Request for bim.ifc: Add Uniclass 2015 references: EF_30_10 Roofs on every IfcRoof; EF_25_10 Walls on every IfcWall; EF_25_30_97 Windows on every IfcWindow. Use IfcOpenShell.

First a look at what the model holds.

```python
import ifcopenshell

model = ifcopenshell.open("bim.ifc")
print(model.schema)
print("classifications:", [c.Name for c in model.by_type("IfcClassification")])
for ifc_class in ("IfcDoor", "IfcRoof", "IfcStair", "IfcWall", "IfcWindow"):
    print(ifc_class, len(model.by_type(ifc_class)))
```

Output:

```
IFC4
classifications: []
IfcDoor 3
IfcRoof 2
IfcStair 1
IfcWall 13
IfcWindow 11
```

```python
import ifcopenshell
import ifcopenshell.api.classification

model = ifcopenshell.open("bim.ifc")

system = ifcopenshell.api.classification.add_classification(model, classification="Uniclass 2015")

codes = {
    "IfcRoof": ("EF_30_10", "Roofs"),
    "IfcWall": ("EF_25_10", "Walls"),
    "IfcWindow": ("EF_25_30_97", "Windows"),
}
for ifc_class, (code, name) in codes.items():
    products = model.by_type(ifc_class)
    ifcopenshell.api.classification.add_reference(
        model, products=products, classification=system, identification=code, name=name
    )
    print(code, len(products))

model.write("bim_rev.ifc")
```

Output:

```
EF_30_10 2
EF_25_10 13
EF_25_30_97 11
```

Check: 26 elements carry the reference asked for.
